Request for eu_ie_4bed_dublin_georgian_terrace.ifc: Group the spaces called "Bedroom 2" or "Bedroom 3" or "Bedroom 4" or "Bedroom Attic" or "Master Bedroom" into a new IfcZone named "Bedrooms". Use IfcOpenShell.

First a look at what the model holds.

```python
import ifcopenshell

model = ifcopenshell.open("eu_ie_4bed_dublin_georgian_terrace.ifc")
print(model.schema)
seen = {}
for space in model.by_type("IfcSpace"):
    seen[space.LongName] = seen.get(space.LongName, 0) + 1
for name, count in sorted(seen.items(), key=str):
    print(count, "x", name)
print("zones:", [z.Name for z in model.by_type("IfcZone")][:20])
```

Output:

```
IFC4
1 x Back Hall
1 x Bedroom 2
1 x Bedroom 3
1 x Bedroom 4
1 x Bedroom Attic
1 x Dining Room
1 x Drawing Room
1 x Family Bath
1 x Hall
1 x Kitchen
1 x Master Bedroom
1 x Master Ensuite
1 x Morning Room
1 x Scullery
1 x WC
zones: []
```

```python
import ifcopenshell
import ifcopenshell.api.group
import ifcopenshell.api.root

model = ifcopenshell.open("eu_ie_4bed_dublin_georgian_terrace.ifc")

names = {"Bedroom 2", "Bedroom 3", "Bedroom 4", "Bedroom Attic", "Master Bedroom"}
spaces = [s for s in model.by_type("IfcSpace") if s.LongName in names]

zone = ifcopenshell.api.root.create_entity(model, ifc_class="IfcZone", name="Bedrooms")
ifcopenshell.api.group.assign_group(model, products=spaces, group=zone)
print(len(spaces), "spaces in", zone.Name)

model.write("eu_ie_4bed_dublin_georgian_terrace-out.ifc")
```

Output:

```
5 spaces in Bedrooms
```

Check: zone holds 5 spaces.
